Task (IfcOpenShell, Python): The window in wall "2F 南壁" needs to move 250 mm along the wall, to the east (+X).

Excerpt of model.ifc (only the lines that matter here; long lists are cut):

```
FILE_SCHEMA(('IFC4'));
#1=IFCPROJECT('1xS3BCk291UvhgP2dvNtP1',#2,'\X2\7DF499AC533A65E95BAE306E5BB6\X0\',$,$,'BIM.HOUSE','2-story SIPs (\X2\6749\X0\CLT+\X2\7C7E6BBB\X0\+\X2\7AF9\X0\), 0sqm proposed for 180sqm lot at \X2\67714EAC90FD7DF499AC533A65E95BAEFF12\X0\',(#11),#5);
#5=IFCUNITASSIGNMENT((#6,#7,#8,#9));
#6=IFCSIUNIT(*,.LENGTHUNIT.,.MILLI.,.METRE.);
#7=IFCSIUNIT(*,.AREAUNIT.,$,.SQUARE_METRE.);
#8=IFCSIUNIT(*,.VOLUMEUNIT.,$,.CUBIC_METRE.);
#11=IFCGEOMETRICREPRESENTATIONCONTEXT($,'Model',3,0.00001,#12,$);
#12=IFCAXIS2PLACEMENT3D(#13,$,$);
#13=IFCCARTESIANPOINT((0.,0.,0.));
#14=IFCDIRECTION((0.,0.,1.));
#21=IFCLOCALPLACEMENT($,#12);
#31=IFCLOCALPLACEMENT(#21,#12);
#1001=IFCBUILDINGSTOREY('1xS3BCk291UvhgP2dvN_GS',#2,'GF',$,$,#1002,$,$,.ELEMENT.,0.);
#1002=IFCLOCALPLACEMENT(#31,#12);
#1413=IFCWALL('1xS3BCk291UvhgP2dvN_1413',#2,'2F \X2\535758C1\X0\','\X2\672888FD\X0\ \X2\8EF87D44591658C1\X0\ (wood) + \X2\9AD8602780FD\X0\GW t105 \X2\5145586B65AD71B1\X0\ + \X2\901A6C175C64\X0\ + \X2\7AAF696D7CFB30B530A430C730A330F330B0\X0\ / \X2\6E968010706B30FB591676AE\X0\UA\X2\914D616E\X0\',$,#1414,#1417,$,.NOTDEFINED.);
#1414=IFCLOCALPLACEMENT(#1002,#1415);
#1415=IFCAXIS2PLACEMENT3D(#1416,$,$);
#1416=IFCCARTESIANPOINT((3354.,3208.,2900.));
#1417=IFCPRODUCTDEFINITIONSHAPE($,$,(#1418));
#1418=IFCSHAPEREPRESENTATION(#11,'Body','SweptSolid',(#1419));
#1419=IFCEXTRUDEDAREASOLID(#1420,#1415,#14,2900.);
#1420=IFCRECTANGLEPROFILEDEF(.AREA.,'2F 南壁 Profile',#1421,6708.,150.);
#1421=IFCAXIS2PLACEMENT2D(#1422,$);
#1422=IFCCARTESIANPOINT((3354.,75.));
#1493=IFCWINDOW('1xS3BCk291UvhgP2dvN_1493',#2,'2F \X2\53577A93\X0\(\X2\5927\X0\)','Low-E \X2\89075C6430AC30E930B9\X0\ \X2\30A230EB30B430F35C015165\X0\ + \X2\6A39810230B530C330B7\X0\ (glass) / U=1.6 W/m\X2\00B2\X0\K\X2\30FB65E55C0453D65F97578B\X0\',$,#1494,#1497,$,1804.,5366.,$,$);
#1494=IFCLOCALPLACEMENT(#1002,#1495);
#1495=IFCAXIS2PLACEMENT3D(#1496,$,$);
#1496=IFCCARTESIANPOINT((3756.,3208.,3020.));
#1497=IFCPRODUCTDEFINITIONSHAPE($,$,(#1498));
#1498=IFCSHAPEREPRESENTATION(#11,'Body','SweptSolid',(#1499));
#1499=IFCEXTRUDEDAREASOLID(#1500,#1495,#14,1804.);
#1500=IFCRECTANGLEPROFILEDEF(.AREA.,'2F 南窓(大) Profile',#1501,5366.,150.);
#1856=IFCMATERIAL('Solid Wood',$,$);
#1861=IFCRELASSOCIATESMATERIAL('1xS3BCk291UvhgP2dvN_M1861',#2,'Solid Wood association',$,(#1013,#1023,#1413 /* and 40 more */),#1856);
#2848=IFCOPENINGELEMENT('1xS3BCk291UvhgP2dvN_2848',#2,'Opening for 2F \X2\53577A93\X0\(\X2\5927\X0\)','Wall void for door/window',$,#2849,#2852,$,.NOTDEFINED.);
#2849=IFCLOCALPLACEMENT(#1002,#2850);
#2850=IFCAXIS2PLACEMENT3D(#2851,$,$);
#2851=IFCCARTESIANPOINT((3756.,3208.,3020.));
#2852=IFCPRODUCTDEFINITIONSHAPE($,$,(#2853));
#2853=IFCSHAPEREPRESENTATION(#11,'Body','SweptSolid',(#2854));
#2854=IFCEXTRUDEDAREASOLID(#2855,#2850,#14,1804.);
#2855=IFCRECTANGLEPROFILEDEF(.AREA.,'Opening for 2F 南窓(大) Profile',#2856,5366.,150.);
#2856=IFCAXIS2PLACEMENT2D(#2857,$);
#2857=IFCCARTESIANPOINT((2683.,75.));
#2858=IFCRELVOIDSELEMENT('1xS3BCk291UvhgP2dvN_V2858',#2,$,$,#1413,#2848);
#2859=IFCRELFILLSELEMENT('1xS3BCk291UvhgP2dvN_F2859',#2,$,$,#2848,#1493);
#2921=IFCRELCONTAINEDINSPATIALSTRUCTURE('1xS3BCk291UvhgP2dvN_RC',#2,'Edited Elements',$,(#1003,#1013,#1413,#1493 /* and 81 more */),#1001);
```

```python
import ifcopenshell
import ifcopenshell.api.geometry
import ifcopenshell.util.placement

model = ifcopenshell.open("model.ifc")

window = model.by_guid("1xS3BCk291UvhgP2dvN_1493")
opening = window.FillsVoids[0].RelatingOpeningElement
wall = opening.VoidsElements[0].RelatingBuildingElement

wall_matrix = ifcopenshell.util.placement.get_local_placement(wall.ObjectPlacement)
shift = wall_matrix[:3, 0] * 250.0
before = ifcopenshell.util.placement.get_local_placement(window.ObjectPlacement)[:3, 3].copy()

# The window is not placed relative to its opening, so move both.
for product in (opening, window):
    matrix = ifcopenshell.util.placement.get_local_placement(product.ObjectPlacement)
    matrix[:3, 3] += shift
    ifcopenshell.api.geometry.edit_object_placement(model, product=product, matrix=matrix, is_si=False)

after = ifcopenshell.util.placement.get_local_placement(window.ObjectPlacement)[:3, 3]
print("window moved by", (after - before).round(3) + 0.0)

model.write("model_rev.ifc")
```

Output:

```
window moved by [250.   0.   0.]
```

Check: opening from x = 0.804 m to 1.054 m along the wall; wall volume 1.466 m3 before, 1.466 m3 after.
